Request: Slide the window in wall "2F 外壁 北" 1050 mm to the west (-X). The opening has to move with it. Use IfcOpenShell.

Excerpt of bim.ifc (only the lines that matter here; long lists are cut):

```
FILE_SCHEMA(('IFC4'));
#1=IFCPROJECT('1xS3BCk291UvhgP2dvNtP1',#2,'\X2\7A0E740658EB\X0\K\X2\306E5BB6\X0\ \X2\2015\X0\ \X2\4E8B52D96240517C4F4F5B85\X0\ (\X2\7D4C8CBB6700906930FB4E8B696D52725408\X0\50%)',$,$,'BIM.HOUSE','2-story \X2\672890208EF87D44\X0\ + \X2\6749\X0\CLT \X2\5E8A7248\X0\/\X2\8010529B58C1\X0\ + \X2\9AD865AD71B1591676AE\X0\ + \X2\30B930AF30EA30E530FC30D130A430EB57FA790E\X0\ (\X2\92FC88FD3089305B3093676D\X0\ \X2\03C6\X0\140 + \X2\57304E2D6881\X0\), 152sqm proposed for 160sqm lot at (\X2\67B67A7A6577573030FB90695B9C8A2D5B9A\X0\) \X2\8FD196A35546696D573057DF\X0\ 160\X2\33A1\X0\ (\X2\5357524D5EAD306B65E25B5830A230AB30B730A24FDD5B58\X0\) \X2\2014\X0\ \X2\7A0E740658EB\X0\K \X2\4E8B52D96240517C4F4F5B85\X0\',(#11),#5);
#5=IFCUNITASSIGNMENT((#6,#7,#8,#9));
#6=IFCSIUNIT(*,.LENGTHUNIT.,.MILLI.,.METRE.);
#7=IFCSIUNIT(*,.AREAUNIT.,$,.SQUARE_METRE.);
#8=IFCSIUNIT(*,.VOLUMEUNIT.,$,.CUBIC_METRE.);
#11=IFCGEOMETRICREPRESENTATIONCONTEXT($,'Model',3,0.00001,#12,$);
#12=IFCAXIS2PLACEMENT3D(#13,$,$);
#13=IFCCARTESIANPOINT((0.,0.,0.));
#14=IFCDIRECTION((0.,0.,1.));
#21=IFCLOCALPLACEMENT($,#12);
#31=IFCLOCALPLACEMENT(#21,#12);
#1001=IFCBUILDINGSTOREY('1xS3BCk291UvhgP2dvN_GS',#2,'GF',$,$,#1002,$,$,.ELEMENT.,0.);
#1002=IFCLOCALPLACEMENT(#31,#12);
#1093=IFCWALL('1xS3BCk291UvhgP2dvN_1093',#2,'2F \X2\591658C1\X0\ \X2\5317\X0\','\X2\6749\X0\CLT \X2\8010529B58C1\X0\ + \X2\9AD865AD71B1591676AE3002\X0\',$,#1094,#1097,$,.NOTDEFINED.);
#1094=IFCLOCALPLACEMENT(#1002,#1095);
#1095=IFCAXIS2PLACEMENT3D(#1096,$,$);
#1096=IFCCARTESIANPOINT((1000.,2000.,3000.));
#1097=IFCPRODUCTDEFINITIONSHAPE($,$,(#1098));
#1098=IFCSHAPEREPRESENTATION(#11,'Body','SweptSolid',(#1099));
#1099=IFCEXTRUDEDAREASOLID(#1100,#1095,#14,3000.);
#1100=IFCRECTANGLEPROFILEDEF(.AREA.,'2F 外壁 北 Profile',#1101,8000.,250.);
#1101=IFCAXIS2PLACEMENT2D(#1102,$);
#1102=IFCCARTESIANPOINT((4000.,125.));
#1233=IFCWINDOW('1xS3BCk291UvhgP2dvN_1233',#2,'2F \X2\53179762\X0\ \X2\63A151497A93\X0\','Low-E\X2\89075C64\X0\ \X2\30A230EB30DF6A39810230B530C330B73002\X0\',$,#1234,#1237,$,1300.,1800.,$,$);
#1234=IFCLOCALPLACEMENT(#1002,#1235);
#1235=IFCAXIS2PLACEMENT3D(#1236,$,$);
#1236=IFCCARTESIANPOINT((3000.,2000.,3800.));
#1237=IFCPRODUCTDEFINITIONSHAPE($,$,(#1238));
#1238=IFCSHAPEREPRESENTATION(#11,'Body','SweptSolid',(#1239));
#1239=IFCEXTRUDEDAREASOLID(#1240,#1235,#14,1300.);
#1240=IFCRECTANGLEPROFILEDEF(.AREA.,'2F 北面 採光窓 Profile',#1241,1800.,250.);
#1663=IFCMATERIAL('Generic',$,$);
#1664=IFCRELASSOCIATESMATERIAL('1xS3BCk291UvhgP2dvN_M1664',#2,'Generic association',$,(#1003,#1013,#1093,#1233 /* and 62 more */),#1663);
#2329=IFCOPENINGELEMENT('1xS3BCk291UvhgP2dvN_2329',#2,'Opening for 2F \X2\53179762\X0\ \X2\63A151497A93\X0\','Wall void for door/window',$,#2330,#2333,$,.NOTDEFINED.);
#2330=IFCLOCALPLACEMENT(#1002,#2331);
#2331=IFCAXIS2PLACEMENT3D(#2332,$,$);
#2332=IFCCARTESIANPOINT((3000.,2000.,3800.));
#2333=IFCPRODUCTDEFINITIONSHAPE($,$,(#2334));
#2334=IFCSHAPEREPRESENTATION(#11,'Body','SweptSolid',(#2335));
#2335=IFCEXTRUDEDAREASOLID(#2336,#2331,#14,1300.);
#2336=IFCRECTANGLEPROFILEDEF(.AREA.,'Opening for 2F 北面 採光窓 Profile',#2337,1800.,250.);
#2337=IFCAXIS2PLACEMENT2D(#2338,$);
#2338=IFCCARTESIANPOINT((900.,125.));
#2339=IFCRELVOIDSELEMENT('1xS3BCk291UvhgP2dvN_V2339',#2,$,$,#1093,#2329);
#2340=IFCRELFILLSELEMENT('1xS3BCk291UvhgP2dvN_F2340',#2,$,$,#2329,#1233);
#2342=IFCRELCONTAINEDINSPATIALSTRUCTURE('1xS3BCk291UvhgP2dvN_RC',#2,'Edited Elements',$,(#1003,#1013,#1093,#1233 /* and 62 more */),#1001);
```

```python
import ifcopenshell
import ifcopenshell.api.geometry
import ifcopenshell.util.placement

model = ifcopenshell.open("bim.ifc")

window = model.by_guid("1xS3BCk291UvhgP2dvN_1233")
opening = window.FillsVoids[0].RelatingOpeningElement
wall = opening.VoidsElements[0].RelatingBuildingElement

wall_matrix = ifcopenshell.util.placement.get_local_placement(wall.ObjectPlacement)
shift = wall_matrix[:3, 0] * -1050.0
before = ifcopenshell.util.placement.get_local_placement(window.ObjectPlacement)[:3, 3].copy()

# The window is not placed relative to its opening, so move both.
for product in (opening, window):
    matrix = ifcopenshell.util.placement.get_local_placement(product.ObjectPlacement)
    matrix[:3, 3] += shift
    ifcopenshell.api.geometry.edit_object_placement(model, product=product, matrix=matrix, is_si=False)

after = ifcopenshell.util.placement.get_local_placement(window.ObjectPlacement)[:3, 3]
print("window moved by", (after - before).round(3) + 0.0)

model.write("bim_updated.ifc")
```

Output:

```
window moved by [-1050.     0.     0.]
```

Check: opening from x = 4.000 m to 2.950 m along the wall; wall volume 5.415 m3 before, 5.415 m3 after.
